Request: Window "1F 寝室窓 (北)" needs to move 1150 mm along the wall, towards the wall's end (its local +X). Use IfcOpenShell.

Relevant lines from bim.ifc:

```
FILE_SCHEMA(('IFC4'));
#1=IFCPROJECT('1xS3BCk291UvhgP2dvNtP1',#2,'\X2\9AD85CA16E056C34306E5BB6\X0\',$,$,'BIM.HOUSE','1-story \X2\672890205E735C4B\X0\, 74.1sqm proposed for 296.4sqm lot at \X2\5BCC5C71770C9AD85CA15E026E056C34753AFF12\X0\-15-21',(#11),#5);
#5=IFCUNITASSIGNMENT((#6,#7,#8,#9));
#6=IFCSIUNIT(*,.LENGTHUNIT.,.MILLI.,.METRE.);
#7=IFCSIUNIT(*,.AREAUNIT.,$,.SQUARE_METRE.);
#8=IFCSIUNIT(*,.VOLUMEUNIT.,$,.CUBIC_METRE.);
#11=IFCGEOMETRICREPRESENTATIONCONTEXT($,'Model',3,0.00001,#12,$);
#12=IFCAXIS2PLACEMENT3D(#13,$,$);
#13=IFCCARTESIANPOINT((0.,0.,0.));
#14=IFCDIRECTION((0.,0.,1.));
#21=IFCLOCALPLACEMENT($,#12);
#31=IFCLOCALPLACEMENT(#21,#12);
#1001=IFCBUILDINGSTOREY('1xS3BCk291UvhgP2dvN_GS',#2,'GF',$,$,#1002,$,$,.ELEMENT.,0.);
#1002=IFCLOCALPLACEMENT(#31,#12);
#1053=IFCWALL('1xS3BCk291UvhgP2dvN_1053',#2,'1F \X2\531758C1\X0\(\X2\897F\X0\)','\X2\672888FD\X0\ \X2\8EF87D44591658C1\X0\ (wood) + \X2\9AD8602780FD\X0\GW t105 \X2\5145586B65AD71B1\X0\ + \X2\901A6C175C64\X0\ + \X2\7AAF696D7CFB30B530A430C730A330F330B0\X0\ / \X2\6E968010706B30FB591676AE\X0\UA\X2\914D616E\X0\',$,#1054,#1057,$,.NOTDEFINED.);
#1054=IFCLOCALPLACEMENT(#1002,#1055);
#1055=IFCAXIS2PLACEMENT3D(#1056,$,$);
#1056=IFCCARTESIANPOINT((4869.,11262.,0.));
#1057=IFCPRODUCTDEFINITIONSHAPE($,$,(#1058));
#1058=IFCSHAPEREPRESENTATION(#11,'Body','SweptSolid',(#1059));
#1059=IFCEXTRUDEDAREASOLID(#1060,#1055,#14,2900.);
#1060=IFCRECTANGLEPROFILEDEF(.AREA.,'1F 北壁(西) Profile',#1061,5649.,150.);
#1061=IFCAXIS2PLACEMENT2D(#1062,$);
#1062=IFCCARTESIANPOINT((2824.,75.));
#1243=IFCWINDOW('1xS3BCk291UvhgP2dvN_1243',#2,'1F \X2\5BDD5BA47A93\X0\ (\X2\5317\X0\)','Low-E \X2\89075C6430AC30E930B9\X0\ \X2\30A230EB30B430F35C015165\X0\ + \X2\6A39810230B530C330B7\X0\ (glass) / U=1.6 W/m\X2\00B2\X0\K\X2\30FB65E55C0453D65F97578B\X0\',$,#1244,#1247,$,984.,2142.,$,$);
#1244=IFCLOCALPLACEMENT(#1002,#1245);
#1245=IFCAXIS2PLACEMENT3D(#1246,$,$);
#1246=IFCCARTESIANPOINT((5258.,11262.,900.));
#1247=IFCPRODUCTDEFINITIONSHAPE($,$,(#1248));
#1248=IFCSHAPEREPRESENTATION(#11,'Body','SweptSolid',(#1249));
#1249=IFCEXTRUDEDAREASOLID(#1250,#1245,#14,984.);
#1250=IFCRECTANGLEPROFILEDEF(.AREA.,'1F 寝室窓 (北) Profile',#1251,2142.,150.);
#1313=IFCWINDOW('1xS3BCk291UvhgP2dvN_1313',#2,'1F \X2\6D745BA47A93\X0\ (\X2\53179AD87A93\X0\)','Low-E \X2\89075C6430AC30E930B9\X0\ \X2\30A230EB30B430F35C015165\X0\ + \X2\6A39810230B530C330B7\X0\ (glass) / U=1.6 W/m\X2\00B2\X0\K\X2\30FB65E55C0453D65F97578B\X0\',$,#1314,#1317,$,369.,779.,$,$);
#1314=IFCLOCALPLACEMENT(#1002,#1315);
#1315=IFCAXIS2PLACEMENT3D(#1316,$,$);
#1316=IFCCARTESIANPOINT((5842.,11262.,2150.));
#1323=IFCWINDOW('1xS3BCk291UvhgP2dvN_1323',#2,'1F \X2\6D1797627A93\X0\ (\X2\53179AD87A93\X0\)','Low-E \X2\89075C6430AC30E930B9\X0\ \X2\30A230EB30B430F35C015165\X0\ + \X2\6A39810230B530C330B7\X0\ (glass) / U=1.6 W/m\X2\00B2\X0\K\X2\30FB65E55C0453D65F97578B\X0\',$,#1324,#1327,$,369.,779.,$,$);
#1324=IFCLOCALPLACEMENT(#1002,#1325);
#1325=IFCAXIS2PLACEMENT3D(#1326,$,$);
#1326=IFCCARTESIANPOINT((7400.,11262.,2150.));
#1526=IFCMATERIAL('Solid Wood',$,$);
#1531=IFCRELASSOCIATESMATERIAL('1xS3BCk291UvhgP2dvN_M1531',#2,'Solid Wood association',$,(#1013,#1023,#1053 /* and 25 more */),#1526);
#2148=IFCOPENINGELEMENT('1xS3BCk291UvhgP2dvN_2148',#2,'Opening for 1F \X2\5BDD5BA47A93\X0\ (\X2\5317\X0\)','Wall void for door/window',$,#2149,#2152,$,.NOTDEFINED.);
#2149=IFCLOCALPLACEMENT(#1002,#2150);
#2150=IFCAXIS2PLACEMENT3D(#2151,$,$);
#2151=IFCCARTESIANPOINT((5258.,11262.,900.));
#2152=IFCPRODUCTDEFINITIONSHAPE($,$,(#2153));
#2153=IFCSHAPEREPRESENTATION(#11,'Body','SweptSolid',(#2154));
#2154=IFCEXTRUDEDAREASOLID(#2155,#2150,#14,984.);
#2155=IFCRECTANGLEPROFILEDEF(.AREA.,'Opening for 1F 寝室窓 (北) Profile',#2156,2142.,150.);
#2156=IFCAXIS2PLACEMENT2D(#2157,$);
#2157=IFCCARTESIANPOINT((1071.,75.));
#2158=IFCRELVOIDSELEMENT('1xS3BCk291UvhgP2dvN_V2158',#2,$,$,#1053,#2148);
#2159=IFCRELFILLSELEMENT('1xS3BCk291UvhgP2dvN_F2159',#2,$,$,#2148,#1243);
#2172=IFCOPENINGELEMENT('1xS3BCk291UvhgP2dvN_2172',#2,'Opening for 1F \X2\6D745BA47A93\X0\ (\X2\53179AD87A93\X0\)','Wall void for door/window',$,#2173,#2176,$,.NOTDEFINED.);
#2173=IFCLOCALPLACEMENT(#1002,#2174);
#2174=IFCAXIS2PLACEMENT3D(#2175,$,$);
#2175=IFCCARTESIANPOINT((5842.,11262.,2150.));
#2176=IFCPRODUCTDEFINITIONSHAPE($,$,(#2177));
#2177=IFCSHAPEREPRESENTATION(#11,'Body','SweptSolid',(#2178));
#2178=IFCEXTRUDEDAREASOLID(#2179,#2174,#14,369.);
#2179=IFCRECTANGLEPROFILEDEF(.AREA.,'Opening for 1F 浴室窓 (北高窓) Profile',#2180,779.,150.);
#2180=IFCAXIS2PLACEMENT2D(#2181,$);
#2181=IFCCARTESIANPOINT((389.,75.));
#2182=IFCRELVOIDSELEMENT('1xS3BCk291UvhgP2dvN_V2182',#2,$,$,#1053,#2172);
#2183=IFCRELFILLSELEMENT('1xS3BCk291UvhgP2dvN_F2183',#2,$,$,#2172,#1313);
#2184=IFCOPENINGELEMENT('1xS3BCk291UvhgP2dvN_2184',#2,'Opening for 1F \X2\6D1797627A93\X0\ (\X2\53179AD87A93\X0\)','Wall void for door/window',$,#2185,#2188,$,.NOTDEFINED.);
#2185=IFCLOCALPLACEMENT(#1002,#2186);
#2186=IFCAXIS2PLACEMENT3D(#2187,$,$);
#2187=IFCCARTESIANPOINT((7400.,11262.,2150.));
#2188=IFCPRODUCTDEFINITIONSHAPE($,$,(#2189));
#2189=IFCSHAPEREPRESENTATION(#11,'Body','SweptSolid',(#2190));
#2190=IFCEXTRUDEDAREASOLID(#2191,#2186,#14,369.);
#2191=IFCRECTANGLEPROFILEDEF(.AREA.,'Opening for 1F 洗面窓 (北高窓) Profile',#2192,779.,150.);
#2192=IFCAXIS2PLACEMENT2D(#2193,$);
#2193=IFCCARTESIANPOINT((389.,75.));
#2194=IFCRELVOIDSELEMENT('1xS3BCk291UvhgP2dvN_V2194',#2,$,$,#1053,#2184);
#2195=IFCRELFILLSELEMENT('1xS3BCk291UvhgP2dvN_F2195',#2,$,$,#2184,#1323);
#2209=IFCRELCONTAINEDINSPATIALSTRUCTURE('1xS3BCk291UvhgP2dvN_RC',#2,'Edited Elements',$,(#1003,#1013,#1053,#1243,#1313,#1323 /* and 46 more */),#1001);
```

```python
import ifcopenshell
import ifcopenshell.api.geometry
import ifcopenshell.util.placement
import ifcopenshell.util.unit

model = ifcopenshell.open("bim.ifc")
unit_scale = ifcopenshell.util.unit.calculate_unit_scale(model)

window = model.by_id(1243)
opening = window.FillsVoids[0].RelatingOpeningElement
wall = opening.VoidsElements[0].RelatingBuildingElement

wall_matrix = ifcopenshell.util.placement.get_local_placement(wall.ObjectPlacement)
shift = wall_matrix[:3, 0] * 1.15 / unit_scale
before = ifcopenshell.util.placement.get_local_placement(window.ObjectPlacement)[:3, 3].copy()

# The window is not placed relative to its opening, so move both.
for product in (opening, window):
    matrix = ifcopenshell.util.placement.get_local_placement(product.ObjectPlacement)
    matrix[:3, 3] += shift
    ifcopenshell.api.geometry.edit_object_placement(model, product=product, matrix=matrix, is_si=False)

after = ifcopenshell.util.placement.get_local_placement(window.ObjectPlacement)[:3, 3]
print("window moved by", (after - before).round(3) + 0.0)

model.write("bim-out.ifc")
```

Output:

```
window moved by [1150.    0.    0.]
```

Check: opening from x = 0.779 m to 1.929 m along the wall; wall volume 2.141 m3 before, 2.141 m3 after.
